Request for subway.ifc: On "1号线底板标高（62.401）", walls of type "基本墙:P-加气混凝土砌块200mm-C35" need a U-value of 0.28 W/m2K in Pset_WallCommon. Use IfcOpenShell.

First a look at what the model holds.

```python
import ifcopenshell
import ifcopenshell.util.element

model = ifcopenshell.open("subway.ifc")
print(model.schema)
storey = next(s for s in model.by_type("IfcBuildingStorey") if s.Name == "1号线底板标高（62.401）")
walls = [e for e in ifcopenshell.util.element.get_decomposition(storey) if e.is_a("IfcWall")]
seen = {}
for e in walls:
    element_type = ifcopenshell.util.element.get_type(e)
    key = (element_type.Name if element_type != e and element_type else None, ifcopenshell.util.element.get_pset(e, "Pset_WallCommon", "ThermalTransmittance"))
    seen[key] = seen.get(key, 0) + 1
for (name, value), count in sorted(seen.items(), key=str):
    print(count, "x", name, "|", value)
```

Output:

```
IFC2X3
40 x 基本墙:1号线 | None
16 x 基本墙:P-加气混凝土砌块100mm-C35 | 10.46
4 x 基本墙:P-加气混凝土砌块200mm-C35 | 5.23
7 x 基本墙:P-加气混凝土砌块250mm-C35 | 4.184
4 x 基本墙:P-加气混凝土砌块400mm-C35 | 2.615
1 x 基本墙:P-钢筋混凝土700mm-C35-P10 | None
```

```python
import ifcopenshell
import ifcopenshell.api.pset
import ifcopenshell.util.element

model = ifcopenshell.open("subway.ifc")

storey = next(s for s in model.by_type("IfcBuildingStorey") if s.Name == "1号线底板标高（62.401）")
walls = [e for e in ifcopenshell.util.element.get_decomposition(storey) if e.is_a("IfcWall")]

count = 0
for e in walls:
    element_type = ifcopenshell.util.element.get_type(e)
    if element_type in (None, e) or element_type.Name != "基本墙:P-加气混凝土砌块200mm-C35":
        continue
    # add_pset returns the element's existing set when there is one.
    pset = ifcopenshell.api.pset.add_pset(model, product=e, name="Pset_WallCommon")
    ifcopenshell.api.pset.edit_pset(model, pset=pset, properties={"ThermalTransmittance": 0.28})
    count += 1

print(count, "walls updated")

model.write("subway-out.ifc")
```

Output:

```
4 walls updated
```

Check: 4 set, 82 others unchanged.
